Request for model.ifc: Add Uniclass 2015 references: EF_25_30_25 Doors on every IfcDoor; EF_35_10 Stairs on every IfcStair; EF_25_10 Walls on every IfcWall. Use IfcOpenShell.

First a look at what the model holds.

```python
import ifcopenshell

model = ifcopenshell.open("model.ifc")
print(model.schema)
print("classifications:", [c.Name for c in model.by_type("IfcClassification")])
for ifc_class in ("IfcDoor", "IfcRoof", "IfcStair", "IfcWall", "IfcWindow"):
    print(ifc_class, len(model.by_type(ifc_class)))
```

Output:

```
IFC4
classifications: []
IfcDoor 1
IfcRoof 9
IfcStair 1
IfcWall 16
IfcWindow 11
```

```python
import ifcopenshell
import ifcopenshell.api.classification

model = ifcopenshell.open("model.ifc")

system = ifcopenshell.api.classification.add_classification(model, classification="Uniclass 2015")

codes = {
    "IfcDoor": ("EF_25_30_25", "Doors"),
    "IfcStair": ("EF_35_10", "Stairs"),
    "IfcWall": ("EF_25_10", "Walls"),
}
for ifc_class, (code, name) in codes.items():
    products = model.by_type(ifc_class)
    ifcopenshell.api.classification.add_reference(
        model, products=products, classification=system, identification=code, name=name
    )
    print(code, len(products))

model.write("model_edited.ifc")
```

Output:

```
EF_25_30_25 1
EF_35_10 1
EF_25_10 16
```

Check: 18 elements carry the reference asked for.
